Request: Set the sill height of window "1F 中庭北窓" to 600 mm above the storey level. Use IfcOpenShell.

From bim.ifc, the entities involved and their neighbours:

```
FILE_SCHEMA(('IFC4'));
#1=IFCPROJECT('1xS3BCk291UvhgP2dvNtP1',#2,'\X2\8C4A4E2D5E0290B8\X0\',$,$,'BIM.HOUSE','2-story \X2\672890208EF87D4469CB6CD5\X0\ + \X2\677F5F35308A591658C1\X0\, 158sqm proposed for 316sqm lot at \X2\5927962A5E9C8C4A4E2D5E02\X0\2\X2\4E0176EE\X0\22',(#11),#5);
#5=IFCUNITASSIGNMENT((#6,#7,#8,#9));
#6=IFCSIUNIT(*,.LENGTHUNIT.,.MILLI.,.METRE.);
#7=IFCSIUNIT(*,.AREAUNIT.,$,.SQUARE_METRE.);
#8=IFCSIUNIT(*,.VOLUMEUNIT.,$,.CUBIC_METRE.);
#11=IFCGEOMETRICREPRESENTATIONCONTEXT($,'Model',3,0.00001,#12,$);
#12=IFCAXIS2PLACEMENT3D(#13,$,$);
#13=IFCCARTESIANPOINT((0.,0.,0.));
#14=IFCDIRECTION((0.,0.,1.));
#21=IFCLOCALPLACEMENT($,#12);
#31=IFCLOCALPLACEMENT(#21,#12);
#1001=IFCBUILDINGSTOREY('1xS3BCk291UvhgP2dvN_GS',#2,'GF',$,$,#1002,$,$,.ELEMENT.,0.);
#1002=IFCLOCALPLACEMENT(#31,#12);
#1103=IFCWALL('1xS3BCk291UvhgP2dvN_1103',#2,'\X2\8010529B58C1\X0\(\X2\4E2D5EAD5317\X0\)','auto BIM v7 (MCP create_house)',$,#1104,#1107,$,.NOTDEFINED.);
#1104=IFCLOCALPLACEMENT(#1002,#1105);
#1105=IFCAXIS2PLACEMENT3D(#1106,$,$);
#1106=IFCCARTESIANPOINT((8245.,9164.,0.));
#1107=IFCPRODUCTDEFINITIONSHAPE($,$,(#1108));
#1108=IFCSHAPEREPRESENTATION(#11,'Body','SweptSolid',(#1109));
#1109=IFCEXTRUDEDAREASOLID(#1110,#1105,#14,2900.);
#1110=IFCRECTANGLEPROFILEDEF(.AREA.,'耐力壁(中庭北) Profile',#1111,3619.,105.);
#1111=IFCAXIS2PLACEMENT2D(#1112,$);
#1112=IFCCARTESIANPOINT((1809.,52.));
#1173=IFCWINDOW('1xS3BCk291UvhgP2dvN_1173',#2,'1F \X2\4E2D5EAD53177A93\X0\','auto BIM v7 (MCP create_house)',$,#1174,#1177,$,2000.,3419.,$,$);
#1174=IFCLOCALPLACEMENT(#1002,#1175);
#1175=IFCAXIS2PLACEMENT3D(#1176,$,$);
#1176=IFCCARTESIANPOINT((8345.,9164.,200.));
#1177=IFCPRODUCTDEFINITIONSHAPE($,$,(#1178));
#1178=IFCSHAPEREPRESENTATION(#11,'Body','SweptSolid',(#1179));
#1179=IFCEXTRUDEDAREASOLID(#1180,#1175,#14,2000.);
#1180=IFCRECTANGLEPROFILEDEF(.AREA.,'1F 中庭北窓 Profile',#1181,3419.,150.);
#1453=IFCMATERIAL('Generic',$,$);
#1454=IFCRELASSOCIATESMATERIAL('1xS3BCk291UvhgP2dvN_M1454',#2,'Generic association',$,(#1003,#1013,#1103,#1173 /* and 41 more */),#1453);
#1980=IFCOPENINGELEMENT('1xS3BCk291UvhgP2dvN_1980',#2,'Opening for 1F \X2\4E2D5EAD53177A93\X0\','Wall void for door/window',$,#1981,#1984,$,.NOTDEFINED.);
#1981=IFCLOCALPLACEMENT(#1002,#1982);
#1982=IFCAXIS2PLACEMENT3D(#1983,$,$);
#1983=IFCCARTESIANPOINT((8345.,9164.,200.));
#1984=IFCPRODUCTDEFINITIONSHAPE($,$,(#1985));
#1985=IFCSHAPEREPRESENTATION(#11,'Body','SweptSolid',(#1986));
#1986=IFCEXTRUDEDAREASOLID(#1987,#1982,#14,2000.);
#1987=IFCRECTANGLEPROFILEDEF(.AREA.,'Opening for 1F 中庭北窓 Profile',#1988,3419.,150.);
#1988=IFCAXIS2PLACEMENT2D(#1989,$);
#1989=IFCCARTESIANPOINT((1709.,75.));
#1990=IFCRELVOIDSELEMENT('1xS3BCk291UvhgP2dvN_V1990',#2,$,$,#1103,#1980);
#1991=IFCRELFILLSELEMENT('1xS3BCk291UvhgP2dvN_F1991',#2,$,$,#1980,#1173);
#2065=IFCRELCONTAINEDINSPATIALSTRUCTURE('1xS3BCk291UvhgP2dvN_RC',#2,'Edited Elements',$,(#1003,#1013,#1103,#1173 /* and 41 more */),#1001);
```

```python
import numpy as np
import ifcopenshell
import ifcopenshell.api.geometry
import ifcopenshell.geom
import ifcopenshell.util.element
import ifcopenshell.util.placement
import ifcopenshell.util.shape
import ifcopenshell.util.unit

model = ifcopenshell.open("bim.ifc")
unit_scale = ifcopenshell.util.unit.calculate_unit_scale(model)

window = model.by_guid("1xS3BCk291UvhgP2dvN_1173")
opening = window.FillsVoids[0].RelatingOpeningElement
storey = ifcopenshell.util.element.get_container(window, ifc_class="IfcBuildingStorey")
level = ifcopenshell.util.placement.get_local_placement(storey.ObjectPlacement)[2, 3]

# The opening's origin need not be at the sill, so measure its lowest point.
shape = ifcopenshell.geom.create_shape(ifcopenshell.geom.settings(), opening)
bottom = ifcopenshell.util.shape.get_shape_bottom_elevation(shape, shape.geometry) / unit_scale
dz = level + 600.0 - bottom

shift = np.array([0.0, 0.0, dz])
# The window is not placed relative to its opening, so move both.
for product in (opening, window):
    matrix = ifcopenshell.util.placement.get_local_placement(product.ObjectPlacement)
    matrix[:3, 3] += shift
    ifcopenshell.api.geometry.edit_object_placement(model, product=product, matrix=matrix, is_si=False)

print(f"moved by {dz * unit_scale:+.3f} m")

model.write("bim_updated.ifc")
```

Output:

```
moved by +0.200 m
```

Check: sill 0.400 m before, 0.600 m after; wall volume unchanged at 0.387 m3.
